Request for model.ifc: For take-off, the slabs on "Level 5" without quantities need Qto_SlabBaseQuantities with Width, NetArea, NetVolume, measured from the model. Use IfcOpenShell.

First a look at what the model holds.

```python
import ifcopenshell
import ifcopenshell.util.element
import ifcopenshell.util.unit

model = ifcopenshell.open("model.ifc")
print(model.schema)
for unit_type in ("LENGTHUNIT", "AREAUNIT", "VOLUMEUNIT"):
    print(unit_type, ifcopenshell.util.unit.calculate_unit_scale(model, unit_type))
storey = next(s for s in model.by_type("IfcBuildingStorey") if s.Name == "Level 5")
slabs = [e for e in ifcopenshell.util.element.get_decomposition(storey) if e.is_a("IfcSlab")]
for e in sorted(slabs, key=lambda e: e.id()):
    print(e.id(), e.is_a(), e.Name, list(ifcopenshell.util.element.get_psets(e, qtos_only=True)), sep=" | ")
```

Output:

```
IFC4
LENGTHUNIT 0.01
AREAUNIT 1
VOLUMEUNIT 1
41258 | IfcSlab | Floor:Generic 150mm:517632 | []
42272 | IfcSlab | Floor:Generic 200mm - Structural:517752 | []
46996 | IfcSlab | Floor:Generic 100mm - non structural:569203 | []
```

```python
import ifcopenshell
import ifcopenshell.api.pset
import ifcopenshell.geom
import ifcopenshell.util.element
import ifcopenshell.util.shape
import ifcopenshell.util.unit

model = ifcopenshell.open("model.ifc")
unit_scale = ifcopenshell.util.unit.calculate_unit_scale(model)
area_scale = ifcopenshell.util.unit.calculate_unit_scale(model, "AREAUNIT")
volume_scale = ifcopenshell.util.unit.calculate_unit_scale(model, "VOLUMEUNIT")
settings = ifcopenshell.geom.settings()

storey = next(s for s in model.by_type("IfcBuildingStorey") if s.Name == "Level 5")
slabs = [e for e in ifcopenshell.util.element.get_decomposition(storey) if e.is_a("IfcSlab")]

for e in sorted(slabs, key=lambda e: e.id()):
    if ifcopenshell.util.element.get_psets(e, qtos_only=True, should_inherit=False):
        continue
    # Geometry comes back in metres, in the element's own axes.
    shape = ifcopenshell.geom.create_shape(settings, e)
    values = {
        "Width": ifcopenshell.util.shape.get_z(shape.geometry) / unit_scale,
        "NetArea": ifcopenshell.util.shape.get_footprint_area(shape.geometry) / area_scale,
        "NetVolume": ifcopenshell.util.shape.get_volume(shape.geometry) / volume_scale,
    }
    qto = ifcopenshell.api.pset.add_qto(model, product=e, name="Qto_SlabBaseQuantities")
    ifcopenshell.api.pset.edit_qto(model, qto=qto, properties=values)
    print(e.id(), {k: round(v, 3) for k, v in values.items()})

model.write("model_updated.ifc")
```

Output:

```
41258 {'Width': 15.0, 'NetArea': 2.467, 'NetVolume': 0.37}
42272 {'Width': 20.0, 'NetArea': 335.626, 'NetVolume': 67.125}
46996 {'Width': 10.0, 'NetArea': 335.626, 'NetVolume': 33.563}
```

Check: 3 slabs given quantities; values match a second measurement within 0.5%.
